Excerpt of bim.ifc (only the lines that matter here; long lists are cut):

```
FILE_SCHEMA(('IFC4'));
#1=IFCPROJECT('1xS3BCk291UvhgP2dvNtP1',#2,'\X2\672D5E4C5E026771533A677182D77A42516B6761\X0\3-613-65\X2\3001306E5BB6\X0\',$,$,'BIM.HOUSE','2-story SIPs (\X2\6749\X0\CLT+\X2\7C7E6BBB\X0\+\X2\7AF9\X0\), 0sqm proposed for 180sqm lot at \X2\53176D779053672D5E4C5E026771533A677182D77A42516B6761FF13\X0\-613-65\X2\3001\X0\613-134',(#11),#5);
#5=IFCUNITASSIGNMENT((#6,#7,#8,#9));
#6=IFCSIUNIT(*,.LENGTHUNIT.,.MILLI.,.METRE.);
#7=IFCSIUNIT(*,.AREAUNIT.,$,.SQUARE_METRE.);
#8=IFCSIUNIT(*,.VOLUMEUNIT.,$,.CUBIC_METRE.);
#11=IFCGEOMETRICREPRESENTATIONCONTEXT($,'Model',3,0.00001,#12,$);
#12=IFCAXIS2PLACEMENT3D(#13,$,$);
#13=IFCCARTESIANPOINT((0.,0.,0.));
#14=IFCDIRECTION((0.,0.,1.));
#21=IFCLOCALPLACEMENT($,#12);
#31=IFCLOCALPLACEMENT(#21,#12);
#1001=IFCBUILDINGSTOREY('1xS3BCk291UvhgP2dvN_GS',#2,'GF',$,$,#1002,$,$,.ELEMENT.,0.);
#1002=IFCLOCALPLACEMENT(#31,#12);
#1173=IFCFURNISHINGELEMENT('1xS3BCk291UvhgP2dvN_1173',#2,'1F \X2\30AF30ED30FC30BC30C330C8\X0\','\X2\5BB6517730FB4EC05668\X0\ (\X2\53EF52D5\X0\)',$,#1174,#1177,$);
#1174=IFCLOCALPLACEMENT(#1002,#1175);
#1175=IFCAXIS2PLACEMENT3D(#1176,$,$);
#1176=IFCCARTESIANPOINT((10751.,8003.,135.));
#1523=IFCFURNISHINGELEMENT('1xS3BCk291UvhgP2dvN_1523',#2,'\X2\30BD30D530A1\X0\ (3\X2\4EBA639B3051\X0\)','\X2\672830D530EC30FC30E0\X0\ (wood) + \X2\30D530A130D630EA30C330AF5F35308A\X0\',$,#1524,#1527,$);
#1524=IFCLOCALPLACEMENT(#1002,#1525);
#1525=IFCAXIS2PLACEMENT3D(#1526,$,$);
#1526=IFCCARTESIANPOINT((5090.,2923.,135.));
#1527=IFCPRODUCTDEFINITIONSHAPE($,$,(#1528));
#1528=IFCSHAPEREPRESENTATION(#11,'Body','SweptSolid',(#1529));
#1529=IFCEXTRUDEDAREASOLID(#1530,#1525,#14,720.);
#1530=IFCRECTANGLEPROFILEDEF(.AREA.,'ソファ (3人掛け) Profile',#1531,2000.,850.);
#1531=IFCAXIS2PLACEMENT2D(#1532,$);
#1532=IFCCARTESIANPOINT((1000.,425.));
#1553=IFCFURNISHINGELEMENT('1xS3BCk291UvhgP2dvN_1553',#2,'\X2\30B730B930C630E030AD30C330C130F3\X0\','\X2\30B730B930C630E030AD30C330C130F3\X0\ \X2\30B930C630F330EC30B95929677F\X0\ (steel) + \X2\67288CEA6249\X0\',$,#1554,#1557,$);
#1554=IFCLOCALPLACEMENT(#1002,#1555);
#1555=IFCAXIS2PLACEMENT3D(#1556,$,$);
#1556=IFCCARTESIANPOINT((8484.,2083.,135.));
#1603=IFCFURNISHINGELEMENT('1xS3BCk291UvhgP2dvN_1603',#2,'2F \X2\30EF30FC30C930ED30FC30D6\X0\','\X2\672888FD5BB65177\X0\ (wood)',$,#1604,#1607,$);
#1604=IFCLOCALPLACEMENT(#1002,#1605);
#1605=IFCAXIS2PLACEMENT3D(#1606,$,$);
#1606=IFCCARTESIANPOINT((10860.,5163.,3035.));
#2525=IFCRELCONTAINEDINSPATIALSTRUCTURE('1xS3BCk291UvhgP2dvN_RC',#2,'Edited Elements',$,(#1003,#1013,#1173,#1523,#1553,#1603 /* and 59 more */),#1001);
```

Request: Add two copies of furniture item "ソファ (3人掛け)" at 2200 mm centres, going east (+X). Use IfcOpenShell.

```python
import numpy as np
import ifcopenshell
import ifcopenshell.api.geometry
import ifcopenshell.api.root
import ifcopenshell.util.element
import ifcopenshell.util.placement
import ifcopenshell.util.unit

model = ifcopenshell.open("bim.ifc")
unit_scale = ifcopenshell.util.unit.calculate_unit_scale(model)


def reuse_history(source, copy):
    """copy_class also copies each property set's owner history, people and application; keep the originals."""
    for rel in copy.IsDefinedBy:
        if rel.is_a("IfcRelDefinesByProperties") and (history := rel.RelatingPropertyDefinition.OwnerHistory):
            rel.RelatingPropertyDefinition.OwnerHistory = source.OwnerHistory
            ifcopenshell.util.element.remove_deep2(model, history)


source = model.by_guid("1xS3BCk291UvhgP2dvN_1523")
base = ifcopenshell.util.placement.get_local_placement(source.ObjectPlacement)
step = np.array([1.0, 0.0, 0.0]) * 2.2 / unit_scale

for i in range(1, 3):
    copy = ifcopenshell.api.root.copy_class(model, product=source)
    copy.Representation = ifcopenshell.util.element.copy_deep(
        model, source.Representation, exclude=["IfcGeometricRepresentationContext", "IfcRepresentationMap"]
    )
    reuse_history(source, copy)
    matrix = base.copy()
    matrix[:3, 3] += i * step
    print("added at", matrix[:3, 3].round(3) + 0.0)
    ifcopenshell.api.geometry.edit_object_placement(model, product=copy, matrix=matrix, is_si=False)

model.write("bim_edited.ifc")
```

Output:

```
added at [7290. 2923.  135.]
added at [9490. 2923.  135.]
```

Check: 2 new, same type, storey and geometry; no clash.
